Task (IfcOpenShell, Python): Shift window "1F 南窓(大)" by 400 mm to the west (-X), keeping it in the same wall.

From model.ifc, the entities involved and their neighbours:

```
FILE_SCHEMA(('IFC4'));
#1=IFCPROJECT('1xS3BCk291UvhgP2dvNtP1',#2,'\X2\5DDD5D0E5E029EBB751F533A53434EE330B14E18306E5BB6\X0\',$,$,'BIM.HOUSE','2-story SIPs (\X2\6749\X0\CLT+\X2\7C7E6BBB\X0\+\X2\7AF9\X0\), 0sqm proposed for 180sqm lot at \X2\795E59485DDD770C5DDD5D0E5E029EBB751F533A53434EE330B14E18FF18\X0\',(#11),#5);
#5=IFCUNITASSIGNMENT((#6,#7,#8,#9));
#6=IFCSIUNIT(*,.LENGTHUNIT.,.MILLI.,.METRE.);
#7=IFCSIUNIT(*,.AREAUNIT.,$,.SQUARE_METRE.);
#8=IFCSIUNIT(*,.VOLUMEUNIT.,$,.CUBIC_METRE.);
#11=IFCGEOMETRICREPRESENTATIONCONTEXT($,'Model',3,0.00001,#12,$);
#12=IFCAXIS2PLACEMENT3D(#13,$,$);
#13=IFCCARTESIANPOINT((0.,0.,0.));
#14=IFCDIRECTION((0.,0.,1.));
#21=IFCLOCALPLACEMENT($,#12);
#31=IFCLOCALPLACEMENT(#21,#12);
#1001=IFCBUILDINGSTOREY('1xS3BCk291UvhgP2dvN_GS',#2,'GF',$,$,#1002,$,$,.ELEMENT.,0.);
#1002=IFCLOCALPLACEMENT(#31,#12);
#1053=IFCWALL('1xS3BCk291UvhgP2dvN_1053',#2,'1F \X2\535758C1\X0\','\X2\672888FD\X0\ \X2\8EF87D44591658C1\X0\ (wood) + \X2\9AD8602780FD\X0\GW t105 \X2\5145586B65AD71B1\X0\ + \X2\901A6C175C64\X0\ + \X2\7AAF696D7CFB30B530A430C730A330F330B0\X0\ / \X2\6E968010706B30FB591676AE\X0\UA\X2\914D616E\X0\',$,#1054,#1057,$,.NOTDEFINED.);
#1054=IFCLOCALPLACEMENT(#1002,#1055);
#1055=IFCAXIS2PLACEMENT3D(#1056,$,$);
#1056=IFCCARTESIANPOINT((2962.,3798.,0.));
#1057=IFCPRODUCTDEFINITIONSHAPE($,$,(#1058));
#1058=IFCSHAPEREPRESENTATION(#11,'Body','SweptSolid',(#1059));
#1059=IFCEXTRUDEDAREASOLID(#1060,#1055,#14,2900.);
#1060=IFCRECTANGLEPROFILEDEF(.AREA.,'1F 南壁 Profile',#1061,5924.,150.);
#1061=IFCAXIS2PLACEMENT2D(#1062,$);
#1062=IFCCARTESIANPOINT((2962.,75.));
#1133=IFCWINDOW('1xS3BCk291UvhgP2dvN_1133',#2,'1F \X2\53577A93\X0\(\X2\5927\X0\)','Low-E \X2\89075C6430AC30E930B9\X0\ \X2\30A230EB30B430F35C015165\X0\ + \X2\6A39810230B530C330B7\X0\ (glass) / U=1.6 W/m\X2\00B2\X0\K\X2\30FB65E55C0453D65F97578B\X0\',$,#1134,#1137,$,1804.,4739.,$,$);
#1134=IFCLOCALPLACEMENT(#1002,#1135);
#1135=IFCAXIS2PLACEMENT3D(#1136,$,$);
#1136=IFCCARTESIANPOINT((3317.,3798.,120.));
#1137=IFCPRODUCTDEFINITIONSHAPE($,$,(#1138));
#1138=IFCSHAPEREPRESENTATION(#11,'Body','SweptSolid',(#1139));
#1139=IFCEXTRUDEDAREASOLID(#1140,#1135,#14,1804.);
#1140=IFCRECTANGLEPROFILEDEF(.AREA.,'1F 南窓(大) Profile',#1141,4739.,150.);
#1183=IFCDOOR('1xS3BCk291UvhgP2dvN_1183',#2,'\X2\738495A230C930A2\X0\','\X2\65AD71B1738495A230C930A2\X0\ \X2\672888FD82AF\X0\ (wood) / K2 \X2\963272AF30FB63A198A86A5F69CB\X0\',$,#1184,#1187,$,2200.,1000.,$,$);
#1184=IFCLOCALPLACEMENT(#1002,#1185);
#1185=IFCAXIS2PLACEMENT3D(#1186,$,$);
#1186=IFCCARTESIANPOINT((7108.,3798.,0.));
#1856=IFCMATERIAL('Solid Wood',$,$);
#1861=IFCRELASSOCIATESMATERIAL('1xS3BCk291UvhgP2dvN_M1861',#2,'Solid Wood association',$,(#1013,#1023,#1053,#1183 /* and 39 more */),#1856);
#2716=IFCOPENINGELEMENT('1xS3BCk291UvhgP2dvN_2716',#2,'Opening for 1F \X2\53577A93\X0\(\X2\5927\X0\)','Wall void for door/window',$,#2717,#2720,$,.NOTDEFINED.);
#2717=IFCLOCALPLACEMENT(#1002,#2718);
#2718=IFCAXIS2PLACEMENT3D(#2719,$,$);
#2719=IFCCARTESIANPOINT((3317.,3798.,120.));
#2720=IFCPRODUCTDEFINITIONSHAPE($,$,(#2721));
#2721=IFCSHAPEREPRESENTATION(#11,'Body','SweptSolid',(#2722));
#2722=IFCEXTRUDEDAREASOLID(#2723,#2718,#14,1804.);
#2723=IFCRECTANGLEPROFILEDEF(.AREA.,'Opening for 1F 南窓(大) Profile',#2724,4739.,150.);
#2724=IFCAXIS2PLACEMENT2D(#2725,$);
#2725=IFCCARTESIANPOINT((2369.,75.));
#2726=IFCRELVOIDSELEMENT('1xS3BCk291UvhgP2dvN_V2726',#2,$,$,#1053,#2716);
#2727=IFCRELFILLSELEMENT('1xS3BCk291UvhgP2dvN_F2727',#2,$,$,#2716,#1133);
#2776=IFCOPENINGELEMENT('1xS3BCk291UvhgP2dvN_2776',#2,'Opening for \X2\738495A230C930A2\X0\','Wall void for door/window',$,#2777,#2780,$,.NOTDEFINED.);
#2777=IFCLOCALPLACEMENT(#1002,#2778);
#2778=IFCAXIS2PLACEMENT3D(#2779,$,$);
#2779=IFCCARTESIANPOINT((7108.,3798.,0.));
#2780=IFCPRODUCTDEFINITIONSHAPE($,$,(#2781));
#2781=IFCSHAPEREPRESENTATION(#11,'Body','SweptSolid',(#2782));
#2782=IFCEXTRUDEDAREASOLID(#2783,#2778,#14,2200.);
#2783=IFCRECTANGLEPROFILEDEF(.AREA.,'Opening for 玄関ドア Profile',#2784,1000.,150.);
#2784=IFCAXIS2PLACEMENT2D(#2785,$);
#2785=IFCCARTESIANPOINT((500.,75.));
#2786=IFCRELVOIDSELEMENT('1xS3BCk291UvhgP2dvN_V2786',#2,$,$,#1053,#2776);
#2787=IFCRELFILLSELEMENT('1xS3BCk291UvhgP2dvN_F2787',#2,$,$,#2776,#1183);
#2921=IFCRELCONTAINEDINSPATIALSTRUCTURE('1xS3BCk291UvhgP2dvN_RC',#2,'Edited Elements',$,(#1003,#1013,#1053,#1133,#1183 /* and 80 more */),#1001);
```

```python
import ifcopenshell
import ifcopenshell.api.geometry
import ifcopenshell.util.placement
import ifcopenshell.util.unit

model = ifcopenshell.open("model.ifc")
unit_scale = ifcopenshell.util.unit.calculate_unit_scale(model)

window = model.by_id(1133)
opening = window.FillsVoids[0].RelatingOpeningElement
wall = opening.VoidsElements[0].RelatingBuildingElement

wall_matrix = ifcopenshell.util.placement.get_local_placement(wall.ObjectPlacement)
shift = wall_matrix[:3, 0] * -0.4 / unit_scale
before = ifcopenshell.util.placement.get_local_placement(window.ObjectPlacement)[:3, 3].copy()

# The window is not placed relative to its opening, so move both.
for product in (opening, window):
    matrix = ifcopenshell.util.placement.get_local_placement(product.ObjectPlacement)
    matrix[:3, 3] += shift
    ifcopenshell.api.geometry.edit_object_placement(model, product=product, matrix=matrix, is_si=False)

after = ifcopenshell.util.placement.get_local_placement(window.ObjectPlacement)[:3, 3]
print("window moved by", (after - before).round(3) + 0.0)

model.write("model_edited.ifc")
```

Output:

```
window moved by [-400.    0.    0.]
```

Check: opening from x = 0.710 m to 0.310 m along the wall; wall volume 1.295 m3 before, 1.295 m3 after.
